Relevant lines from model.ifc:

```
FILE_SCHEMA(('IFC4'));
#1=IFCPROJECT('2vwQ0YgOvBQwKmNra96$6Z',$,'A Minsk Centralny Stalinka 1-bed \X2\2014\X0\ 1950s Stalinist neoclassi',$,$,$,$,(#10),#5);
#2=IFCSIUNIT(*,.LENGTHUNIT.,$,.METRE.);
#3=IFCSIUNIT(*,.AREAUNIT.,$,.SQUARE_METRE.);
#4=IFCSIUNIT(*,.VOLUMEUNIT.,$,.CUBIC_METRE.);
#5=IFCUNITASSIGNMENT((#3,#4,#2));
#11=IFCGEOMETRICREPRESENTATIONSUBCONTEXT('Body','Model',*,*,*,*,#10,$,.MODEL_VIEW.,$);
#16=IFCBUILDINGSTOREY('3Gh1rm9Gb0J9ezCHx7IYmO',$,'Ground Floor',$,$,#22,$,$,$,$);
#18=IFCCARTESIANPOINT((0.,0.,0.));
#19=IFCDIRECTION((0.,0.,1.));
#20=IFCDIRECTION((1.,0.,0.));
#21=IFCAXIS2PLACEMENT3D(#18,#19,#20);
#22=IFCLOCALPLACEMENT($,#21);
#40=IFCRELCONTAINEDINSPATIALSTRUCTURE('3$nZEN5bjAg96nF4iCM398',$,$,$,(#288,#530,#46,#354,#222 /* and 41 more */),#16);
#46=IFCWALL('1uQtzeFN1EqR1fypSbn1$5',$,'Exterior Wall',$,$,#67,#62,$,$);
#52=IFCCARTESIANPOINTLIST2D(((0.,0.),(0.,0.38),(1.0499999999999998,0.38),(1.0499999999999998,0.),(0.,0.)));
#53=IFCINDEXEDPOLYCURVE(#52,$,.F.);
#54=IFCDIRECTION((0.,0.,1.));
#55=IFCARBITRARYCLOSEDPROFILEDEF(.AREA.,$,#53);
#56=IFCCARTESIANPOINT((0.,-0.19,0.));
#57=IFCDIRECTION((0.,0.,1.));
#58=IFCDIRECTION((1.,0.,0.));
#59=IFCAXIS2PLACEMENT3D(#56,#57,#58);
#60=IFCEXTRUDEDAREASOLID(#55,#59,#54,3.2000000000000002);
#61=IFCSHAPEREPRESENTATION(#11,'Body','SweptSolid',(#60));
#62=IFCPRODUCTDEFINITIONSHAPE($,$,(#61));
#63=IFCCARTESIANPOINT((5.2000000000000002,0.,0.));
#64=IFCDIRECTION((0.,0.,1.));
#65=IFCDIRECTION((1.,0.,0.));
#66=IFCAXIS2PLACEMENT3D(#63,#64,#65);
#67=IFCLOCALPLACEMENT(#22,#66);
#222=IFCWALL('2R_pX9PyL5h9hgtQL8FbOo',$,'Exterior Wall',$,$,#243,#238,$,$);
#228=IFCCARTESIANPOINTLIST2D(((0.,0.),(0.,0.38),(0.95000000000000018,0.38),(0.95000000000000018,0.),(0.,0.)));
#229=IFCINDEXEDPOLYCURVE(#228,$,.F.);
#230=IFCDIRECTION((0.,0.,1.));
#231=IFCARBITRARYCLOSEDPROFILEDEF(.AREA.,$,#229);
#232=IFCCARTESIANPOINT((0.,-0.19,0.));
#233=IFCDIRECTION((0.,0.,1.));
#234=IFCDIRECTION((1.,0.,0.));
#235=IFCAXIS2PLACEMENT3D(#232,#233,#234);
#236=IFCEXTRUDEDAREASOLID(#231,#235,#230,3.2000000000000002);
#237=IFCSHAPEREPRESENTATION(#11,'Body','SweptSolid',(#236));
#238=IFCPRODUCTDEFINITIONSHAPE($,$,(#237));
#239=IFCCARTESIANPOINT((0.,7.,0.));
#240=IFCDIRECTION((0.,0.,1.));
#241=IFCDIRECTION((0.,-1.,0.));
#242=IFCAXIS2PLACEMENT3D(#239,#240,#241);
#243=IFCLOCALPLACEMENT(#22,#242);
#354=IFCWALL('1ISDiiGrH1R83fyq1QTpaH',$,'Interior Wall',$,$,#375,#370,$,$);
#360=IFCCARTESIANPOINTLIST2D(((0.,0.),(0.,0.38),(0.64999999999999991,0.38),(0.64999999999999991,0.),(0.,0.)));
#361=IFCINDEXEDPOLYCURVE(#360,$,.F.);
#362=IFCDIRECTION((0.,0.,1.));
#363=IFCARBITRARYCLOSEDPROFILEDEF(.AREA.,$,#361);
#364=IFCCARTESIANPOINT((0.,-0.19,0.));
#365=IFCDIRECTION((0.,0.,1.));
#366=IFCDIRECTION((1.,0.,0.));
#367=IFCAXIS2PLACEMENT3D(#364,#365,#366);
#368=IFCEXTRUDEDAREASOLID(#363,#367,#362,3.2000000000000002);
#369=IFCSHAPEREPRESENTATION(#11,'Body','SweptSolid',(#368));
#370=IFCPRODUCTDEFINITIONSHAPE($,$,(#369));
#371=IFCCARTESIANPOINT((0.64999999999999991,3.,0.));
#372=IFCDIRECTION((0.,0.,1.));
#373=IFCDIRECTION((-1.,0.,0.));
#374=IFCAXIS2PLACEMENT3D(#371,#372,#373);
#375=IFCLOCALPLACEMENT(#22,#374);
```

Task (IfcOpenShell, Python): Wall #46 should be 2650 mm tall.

```python
import ifcopenshell
import ifcopenshell.geom
import ifcopenshell.util.representation
import ifcopenshell.util.shape

model = ifcopenshell.open("model.ifc")
settings = ifcopenshell.geom.settings()


def volume(element):
    """Net volume in cubic metres, openings subtracted."""
    shape = ifcopenshell.geom.create_shape(settings, element)
    return ifcopenshell.util.shape.get_volume(shape.geometry)


wall = model.by_guid("1uQtzeFN1EqR1fypSbn1$5")
before = volume(wall)

body = ifcopenshell.util.representation.get_representation(wall, "Model", "Body")
solid = body.Items[0]
old_height = solid.Depth
solid.Depth = 2.65
after = volume(wall)

print(f"height {old_height:g} -> {solid.Depth:g}, volume {before:.3f} -> {after:.3f} m3")

model.write("model_updated.ifc")
```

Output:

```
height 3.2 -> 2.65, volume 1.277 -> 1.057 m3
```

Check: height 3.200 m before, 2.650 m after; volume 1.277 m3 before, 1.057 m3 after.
